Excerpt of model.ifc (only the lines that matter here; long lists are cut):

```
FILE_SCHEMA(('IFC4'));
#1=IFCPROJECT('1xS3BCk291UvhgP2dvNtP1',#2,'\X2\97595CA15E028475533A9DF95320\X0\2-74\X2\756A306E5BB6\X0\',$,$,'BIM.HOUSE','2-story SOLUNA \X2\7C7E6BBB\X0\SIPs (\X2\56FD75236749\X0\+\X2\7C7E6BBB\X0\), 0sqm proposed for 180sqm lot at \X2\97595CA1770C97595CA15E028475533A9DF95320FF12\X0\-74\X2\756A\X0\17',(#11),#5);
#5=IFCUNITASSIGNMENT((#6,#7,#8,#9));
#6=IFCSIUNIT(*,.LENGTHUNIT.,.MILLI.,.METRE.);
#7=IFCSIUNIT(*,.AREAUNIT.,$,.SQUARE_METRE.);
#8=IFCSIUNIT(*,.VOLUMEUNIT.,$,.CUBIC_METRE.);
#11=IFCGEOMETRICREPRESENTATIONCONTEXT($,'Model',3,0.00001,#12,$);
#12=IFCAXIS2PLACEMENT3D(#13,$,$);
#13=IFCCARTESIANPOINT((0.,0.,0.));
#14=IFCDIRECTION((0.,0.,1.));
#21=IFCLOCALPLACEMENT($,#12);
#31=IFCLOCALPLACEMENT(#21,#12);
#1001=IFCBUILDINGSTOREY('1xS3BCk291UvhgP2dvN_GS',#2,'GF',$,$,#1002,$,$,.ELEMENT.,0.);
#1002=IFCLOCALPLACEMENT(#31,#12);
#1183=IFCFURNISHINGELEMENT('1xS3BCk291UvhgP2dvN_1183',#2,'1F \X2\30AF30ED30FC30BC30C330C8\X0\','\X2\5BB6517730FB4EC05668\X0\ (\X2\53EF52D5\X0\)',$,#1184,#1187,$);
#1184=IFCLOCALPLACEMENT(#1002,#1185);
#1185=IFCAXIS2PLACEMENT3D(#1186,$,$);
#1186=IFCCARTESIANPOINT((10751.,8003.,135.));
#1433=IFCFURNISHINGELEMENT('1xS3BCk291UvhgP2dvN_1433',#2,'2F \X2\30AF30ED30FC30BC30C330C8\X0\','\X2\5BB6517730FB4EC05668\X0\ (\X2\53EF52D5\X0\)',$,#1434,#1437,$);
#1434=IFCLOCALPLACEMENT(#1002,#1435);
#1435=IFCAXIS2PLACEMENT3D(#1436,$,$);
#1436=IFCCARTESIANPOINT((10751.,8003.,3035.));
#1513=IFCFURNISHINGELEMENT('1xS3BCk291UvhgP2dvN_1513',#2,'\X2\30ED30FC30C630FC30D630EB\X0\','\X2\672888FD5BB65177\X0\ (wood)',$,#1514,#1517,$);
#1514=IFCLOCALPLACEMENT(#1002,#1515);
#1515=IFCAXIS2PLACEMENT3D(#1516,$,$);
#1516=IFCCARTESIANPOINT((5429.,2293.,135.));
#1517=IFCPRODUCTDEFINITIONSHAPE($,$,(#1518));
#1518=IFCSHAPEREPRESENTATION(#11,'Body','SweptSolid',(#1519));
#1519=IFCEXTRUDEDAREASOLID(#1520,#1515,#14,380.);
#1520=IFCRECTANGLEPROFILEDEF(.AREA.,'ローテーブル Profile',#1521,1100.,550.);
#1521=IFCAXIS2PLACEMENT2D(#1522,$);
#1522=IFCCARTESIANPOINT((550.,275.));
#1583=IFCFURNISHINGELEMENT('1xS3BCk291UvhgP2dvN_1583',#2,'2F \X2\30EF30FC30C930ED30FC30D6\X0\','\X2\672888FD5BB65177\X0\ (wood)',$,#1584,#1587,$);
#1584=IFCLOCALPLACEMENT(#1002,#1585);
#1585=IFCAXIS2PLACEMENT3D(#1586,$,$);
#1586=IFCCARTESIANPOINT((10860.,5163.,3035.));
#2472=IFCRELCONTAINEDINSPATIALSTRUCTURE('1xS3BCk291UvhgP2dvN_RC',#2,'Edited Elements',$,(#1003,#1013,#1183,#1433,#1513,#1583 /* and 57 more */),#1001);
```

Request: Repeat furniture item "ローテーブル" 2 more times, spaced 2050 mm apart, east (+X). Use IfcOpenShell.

```python
import numpy as np
import ifcopenshell
import ifcopenshell.api.geometry
import ifcopenshell.api.root
import ifcopenshell.util.element
import ifcopenshell.util.placement
import ifcopenshell.util.unit

model = ifcopenshell.open("model.ifc")
unit_scale = ifcopenshell.util.unit.calculate_unit_scale(model)


def reuse_history(source, copy):
    """copy_class also copies each property set's owner history, people and application; keep the originals."""
    for rel in copy.IsDefinedBy:
        if rel.is_a("IfcRelDefinesByProperties") and (history := rel.RelatingPropertyDefinition.OwnerHistory):
            rel.RelatingPropertyDefinition.OwnerHistory = source.OwnerHistory
            ifcopenshell.util.element.remove_deep2(model, history)


source = model.by_guid("1xS3BCk291UvhgP2dvN_1513")
base = ifcopenshell.util.placement.get_local_placement(source.ObjectPlacement)
step = np.array([1.0, 0.0, 0.0]) * 2.05 / unit_scale

for i in range(1, 3):
    copy = ifcopenshell.api.root.copy_class(model, product=source)
    copy.Representation = ifcopenshell.util.element.copy_deep(
        model, source.Representation, exclude=["IfcGeometricRepresentationContext", "IfcRepresentationMap"]
    )
    reuse_history(source, copy)
    matrix = base.copy()
    matrix[:3, 3] += i * step
    print("added at", matrix[:3, 3].round(3) + 0.0)
    ifcopenshell.api.geometry.edit_object_placement(model, product=copy, matrix=matrix, is_si=False)

model.write("model-out.ifc")
```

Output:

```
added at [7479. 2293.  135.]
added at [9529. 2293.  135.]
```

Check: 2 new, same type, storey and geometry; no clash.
